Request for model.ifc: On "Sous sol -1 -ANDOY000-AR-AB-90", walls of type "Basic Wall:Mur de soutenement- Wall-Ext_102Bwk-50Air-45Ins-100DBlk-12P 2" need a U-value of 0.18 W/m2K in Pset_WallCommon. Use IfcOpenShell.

First a look at what the model holds.

```python
import ifcopenshell
import ifcopenshell.util.element

model = ifcopenshell.open("model.ifc")
print(model.schema)
storey = next(s for s in model.by_type("IfcBuildingStorey") if s.Name == "Sous sol -1 -ANDOY000-AR-AB-90")
walls = [e for e in ifcopenshell.util.element.get_decomposition(storey) if e.is_a("IfcWall")]
seen = {}
for e in walls:
    element_type = ifcopenshell.util.element.get_type(e)
    key = (element_type.Name if element_type != e and element_type else None, ifcopenshell.util.element.get_pset(e, "Pset_WallCommon", "ThermalTransmittance"))
    seen[key] = seen.get(key, 0) + 1
for (name, value), count in sorted(seen.items(), key=str):
    print(count, "x", name, "|", value)
```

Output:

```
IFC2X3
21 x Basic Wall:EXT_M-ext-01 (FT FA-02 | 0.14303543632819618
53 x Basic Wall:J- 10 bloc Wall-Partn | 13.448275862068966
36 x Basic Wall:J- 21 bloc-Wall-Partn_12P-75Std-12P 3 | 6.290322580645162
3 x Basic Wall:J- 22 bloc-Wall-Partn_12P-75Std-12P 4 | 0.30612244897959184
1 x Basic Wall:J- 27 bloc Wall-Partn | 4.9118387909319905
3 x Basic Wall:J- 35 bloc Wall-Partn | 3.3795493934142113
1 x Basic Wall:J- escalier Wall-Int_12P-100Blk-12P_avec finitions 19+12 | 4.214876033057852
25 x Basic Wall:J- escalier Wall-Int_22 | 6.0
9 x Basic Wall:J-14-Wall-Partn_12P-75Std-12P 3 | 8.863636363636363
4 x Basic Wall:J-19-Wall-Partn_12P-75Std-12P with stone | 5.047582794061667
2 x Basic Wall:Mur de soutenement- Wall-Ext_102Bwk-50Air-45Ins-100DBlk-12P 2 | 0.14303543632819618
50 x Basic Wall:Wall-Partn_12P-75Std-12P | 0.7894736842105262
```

```python
import ifcopenshell
import ifcopenshell.api.pset
import ifcopenshell.util.element

model = ifcopenshell.open("model.ifc")

storey = next(s for s in model.by_type("IfcBuildingStorey") if s.Name == "Sous sol -1 -ANDOY000-AR-AB-90")
walls = [e for e in ifcopenshell.util.element.get_decomposition(storey) if e.is_a("IfcWall")]

count = 0
for e in walls:
    element_type = ifcopenshell.util.element.get_type(e)
    if element_type in (None, e) or element_type.Name != "Basic Wall:Mur de soutenement- Wall-Ext_102Bwk-50Air-45Ins-100DBlk-12P 2":
        continue
    # add_pset returns the element's existing set when there is one.
    pset = ifcopenshell.api.pset.add_pset(model, product=e, name="Pset_WallCommon")
    ifcopenshell.api.pset.edit_pset(model, pset=pset, properties={"ThermalTransmittance": 0.18})
    count += 1

print(count, "walls updated")

model.write("model_updated.ifc")
```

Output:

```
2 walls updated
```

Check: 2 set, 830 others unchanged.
